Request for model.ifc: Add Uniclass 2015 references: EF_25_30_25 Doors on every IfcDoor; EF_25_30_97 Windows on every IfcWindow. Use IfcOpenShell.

First a look at what the model holds.

```python
import ifcopenshell

model = ifcopenshell.open("model.ifc")
print(model.schema)
print("classifications:", [c.Name for c in model.by_type("IfcClassification")])
for ifc_class in ("IfcDoor", "IfcRoof", "IfcStair", "IfcWall", "IfcWindow"):
    print(ifc_class, len(model.by_type(ifc_class)))
```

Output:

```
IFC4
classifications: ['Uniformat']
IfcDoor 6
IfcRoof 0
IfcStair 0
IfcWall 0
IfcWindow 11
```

```python
import ifcopenshell
import ifcopenshell.api.classification

model = ifcopenshell.open("model.ifc")

system = ifcopenshell.api.classification.add_classification(model, classification="Uniclass 2015")

codes = {
    "IfcDoor": ("EF_25_30_25", "Doors"),
    "IfcWindow": ("EF_25_30_97", "Windows"),
}
for ifc_class, (code, name) in codes.items():
    products = model.by_type(ifc_class)
    ifcopenshell.api.classification.add_reference(
        model, products=products, classification=system, identification=code, name=name
    )
    print(code, len(products))

model.write("model_v2.ifc")
```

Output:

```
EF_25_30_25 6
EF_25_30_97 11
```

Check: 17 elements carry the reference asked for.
